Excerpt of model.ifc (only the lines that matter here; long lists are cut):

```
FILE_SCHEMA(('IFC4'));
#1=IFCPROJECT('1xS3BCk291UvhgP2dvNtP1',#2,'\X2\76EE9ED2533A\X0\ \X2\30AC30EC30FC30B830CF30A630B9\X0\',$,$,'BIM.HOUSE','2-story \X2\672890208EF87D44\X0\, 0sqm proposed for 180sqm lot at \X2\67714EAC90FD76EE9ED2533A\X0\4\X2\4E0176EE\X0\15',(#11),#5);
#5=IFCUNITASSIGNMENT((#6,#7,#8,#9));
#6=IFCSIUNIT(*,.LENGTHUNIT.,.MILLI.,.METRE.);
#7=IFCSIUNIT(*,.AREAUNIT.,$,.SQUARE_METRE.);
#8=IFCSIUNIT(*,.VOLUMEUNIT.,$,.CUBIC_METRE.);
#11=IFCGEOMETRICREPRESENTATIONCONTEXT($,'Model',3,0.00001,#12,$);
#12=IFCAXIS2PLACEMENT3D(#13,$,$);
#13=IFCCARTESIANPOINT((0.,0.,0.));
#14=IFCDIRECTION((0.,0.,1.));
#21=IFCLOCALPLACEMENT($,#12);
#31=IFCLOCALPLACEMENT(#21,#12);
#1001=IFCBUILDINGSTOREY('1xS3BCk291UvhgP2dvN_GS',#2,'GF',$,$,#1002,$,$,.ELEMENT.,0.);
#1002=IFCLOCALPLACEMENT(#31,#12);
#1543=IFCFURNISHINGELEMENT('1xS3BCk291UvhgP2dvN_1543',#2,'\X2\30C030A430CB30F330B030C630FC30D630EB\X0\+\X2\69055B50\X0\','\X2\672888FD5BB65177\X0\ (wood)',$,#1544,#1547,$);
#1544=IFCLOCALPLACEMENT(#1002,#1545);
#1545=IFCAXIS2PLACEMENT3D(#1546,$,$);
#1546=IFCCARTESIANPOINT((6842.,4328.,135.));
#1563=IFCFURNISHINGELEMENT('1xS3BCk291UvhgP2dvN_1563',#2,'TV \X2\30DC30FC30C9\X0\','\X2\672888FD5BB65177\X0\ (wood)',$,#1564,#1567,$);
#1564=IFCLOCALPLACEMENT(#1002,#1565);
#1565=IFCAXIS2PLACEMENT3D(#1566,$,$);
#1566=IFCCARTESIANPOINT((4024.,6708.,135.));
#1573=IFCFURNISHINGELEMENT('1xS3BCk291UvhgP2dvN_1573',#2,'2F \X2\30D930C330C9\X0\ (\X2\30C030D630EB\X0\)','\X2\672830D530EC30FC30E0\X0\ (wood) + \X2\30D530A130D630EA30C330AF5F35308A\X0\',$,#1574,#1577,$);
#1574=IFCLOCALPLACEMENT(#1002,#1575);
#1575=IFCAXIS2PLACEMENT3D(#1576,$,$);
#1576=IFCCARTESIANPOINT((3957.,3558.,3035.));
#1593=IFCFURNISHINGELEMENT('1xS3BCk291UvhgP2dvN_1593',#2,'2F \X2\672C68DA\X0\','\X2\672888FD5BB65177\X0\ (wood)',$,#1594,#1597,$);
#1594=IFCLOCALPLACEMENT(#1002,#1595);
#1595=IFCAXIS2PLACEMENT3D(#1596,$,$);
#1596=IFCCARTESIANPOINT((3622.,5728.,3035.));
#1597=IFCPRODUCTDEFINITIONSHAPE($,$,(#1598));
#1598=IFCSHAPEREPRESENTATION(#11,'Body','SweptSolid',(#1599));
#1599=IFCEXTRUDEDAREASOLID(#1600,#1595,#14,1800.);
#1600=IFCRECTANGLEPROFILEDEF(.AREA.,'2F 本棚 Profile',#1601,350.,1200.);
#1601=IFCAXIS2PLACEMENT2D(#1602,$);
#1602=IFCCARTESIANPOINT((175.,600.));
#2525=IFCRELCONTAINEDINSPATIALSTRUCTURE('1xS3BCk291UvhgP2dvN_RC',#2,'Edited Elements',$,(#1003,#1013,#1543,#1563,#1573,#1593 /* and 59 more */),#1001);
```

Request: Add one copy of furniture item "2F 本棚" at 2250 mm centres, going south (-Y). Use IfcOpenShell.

```python
import numpy as np
import ifcopenshell
import ifcopenshell.api.geometry
import ifcopenshell.api.root
import ifcopenshell.util.element
import ifcopenshell.util.placement
import ifcopenshell.util.unit

model = ifcopenshell.open("model.ifc")
unit_scale = ifcopenshell.util.unit.calculate_unit_scale(model)


def reuse_history(source, copy):
    """copy_class also copies each property set's owner history, people and application; keep the originals."""
    for rel in copy.IsDefinedBy:
        if rel.is_a("IfcRelDefinesByProperties") and (history := rel.RelatingPropertyDefinition.OwnerHistory):
            rel.RelatingPropertyDefinition.OwnerHistory = source.OwnerHistory
            ifcopenshell.util.element.remove_deep2(model, history)


source = model.by_guid("1xS3BCk291UvhgP2dvN_1593")
base = ifcopenshell.util.placement.get_local_placement(source.ObjectPlacement)
step = np.array([0.0, -1.0, 0.0]) * 2.25 / unit_scale

for i in range(1, 2):
    copy = ifcopenshell.api.root.copy_class(model, product=source)
    copy.Representation = ifcopenshell.util.element.copy_deep(
        model, source.Representation, exclude=["IfcGeometricRepresentationContext", "IfcRepresentationMap"]
    )
    reuse_history(source, copy)
    matrix = base.copy()
    matrix[:3, 3] += i * step
    print("added at", matrix[:3, 3].round(3) + 0.0)
    ifcopenshell.api.geometry.edit_object_placement(model, product=copy, matrix=matrix, is_si=False)

model.write("model_edited.ifc")
```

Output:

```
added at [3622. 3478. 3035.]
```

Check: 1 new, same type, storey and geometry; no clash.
